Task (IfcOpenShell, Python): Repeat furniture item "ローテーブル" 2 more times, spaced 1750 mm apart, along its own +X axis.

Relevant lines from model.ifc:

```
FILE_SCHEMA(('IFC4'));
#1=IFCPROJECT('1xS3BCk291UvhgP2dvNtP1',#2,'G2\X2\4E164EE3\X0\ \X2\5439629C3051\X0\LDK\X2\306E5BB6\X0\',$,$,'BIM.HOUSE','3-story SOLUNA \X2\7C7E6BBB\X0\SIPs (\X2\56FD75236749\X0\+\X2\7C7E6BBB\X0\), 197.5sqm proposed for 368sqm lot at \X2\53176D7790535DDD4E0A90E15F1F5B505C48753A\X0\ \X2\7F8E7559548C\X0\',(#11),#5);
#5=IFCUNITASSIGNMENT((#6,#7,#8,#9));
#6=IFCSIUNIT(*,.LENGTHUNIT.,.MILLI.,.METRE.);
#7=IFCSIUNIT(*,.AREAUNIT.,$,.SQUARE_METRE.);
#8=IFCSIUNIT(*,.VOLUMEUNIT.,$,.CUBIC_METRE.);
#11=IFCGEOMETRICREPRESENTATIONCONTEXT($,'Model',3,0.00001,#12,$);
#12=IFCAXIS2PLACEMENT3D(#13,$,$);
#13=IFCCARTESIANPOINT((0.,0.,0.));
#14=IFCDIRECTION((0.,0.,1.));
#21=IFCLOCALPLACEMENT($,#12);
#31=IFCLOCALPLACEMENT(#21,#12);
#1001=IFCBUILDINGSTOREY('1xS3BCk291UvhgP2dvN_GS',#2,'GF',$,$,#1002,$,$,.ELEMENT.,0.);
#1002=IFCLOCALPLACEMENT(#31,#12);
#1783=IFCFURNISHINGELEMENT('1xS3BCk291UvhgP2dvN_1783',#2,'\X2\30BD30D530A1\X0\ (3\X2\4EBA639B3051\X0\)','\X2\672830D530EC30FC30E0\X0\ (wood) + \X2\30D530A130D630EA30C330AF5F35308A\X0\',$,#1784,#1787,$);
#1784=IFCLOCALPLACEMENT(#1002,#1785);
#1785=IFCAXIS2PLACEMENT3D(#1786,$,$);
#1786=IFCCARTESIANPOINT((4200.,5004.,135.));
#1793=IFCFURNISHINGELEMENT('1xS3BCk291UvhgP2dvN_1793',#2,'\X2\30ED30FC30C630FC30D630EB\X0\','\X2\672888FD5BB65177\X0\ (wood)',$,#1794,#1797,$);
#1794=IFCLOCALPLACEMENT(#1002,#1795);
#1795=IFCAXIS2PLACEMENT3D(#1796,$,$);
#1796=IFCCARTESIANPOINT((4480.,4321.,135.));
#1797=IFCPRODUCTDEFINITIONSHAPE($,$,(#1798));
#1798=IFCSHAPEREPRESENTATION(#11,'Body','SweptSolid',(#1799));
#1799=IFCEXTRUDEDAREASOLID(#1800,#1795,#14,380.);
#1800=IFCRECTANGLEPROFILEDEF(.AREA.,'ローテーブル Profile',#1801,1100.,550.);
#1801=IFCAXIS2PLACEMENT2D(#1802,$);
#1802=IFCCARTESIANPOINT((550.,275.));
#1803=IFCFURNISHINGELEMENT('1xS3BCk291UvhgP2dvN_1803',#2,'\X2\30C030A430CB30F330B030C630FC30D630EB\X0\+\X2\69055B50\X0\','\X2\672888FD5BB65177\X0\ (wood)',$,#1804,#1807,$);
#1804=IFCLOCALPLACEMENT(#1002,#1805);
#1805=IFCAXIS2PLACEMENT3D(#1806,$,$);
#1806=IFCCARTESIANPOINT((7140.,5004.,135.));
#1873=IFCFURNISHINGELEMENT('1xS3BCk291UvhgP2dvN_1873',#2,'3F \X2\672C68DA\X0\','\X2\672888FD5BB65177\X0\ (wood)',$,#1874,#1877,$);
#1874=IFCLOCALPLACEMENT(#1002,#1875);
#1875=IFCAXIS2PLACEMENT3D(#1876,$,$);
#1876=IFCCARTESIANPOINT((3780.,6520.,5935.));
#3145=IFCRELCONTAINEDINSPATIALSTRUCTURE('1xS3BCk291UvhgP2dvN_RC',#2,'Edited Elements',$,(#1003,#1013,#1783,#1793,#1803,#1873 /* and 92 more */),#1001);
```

```python
import ifcopenshell
import ifcopenshell.api.geometry
import ifcopenshell.api.root
import ifcopenshell.util.element
import ifcopenshell.util.placement

model = ifcopenshell.open("model.ifc")


def reuse_history(source, copy):
    """copy_class also copies each property set's owner history, people and application; keep the originals."""
    for rel in copy.IsDefinedBy:
        if rel.is_a("IfcRelDefinesByProperties") and (history := rel.RelatingPropertyDefinition.OwnerHistory):
            rel.RelatingPropertyDefinition.OwnerHistory = source.OwnerHistory
            ifcopenshell.util.element.remove_deep2(model, history)


source = model.by_guid("1xS3BCk291UvhgP2dvN_1793")
base = ifcopenshell.util.placement.get_local_placement(source.ObjectPlacement)
step = base[:3, 0] * 1750.0

for i in range(1, 3):
    copy = ifcopenshell.api.root.copy_class(model, product=source)
    copy.Representation = ifcopenshell.util.element.copy_deep(
        model, source.Representation, exclude=["IfcGeometricRepresentationContext", "IfcRepresentationMap"]
    )
    reuse_history(source, copy)
    matrix = base.copy()
    matrix[:3, 3] += i * step
    print("added at", matrix[:3, 3].round(3) + 0.0)
    ifcopenshell.api.geometry.edit_object_placement(model, product=copy, matrix=matrix, is_si=False)

model.write("model_rev.ifc")
```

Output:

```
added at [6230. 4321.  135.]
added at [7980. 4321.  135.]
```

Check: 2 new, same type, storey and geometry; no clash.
